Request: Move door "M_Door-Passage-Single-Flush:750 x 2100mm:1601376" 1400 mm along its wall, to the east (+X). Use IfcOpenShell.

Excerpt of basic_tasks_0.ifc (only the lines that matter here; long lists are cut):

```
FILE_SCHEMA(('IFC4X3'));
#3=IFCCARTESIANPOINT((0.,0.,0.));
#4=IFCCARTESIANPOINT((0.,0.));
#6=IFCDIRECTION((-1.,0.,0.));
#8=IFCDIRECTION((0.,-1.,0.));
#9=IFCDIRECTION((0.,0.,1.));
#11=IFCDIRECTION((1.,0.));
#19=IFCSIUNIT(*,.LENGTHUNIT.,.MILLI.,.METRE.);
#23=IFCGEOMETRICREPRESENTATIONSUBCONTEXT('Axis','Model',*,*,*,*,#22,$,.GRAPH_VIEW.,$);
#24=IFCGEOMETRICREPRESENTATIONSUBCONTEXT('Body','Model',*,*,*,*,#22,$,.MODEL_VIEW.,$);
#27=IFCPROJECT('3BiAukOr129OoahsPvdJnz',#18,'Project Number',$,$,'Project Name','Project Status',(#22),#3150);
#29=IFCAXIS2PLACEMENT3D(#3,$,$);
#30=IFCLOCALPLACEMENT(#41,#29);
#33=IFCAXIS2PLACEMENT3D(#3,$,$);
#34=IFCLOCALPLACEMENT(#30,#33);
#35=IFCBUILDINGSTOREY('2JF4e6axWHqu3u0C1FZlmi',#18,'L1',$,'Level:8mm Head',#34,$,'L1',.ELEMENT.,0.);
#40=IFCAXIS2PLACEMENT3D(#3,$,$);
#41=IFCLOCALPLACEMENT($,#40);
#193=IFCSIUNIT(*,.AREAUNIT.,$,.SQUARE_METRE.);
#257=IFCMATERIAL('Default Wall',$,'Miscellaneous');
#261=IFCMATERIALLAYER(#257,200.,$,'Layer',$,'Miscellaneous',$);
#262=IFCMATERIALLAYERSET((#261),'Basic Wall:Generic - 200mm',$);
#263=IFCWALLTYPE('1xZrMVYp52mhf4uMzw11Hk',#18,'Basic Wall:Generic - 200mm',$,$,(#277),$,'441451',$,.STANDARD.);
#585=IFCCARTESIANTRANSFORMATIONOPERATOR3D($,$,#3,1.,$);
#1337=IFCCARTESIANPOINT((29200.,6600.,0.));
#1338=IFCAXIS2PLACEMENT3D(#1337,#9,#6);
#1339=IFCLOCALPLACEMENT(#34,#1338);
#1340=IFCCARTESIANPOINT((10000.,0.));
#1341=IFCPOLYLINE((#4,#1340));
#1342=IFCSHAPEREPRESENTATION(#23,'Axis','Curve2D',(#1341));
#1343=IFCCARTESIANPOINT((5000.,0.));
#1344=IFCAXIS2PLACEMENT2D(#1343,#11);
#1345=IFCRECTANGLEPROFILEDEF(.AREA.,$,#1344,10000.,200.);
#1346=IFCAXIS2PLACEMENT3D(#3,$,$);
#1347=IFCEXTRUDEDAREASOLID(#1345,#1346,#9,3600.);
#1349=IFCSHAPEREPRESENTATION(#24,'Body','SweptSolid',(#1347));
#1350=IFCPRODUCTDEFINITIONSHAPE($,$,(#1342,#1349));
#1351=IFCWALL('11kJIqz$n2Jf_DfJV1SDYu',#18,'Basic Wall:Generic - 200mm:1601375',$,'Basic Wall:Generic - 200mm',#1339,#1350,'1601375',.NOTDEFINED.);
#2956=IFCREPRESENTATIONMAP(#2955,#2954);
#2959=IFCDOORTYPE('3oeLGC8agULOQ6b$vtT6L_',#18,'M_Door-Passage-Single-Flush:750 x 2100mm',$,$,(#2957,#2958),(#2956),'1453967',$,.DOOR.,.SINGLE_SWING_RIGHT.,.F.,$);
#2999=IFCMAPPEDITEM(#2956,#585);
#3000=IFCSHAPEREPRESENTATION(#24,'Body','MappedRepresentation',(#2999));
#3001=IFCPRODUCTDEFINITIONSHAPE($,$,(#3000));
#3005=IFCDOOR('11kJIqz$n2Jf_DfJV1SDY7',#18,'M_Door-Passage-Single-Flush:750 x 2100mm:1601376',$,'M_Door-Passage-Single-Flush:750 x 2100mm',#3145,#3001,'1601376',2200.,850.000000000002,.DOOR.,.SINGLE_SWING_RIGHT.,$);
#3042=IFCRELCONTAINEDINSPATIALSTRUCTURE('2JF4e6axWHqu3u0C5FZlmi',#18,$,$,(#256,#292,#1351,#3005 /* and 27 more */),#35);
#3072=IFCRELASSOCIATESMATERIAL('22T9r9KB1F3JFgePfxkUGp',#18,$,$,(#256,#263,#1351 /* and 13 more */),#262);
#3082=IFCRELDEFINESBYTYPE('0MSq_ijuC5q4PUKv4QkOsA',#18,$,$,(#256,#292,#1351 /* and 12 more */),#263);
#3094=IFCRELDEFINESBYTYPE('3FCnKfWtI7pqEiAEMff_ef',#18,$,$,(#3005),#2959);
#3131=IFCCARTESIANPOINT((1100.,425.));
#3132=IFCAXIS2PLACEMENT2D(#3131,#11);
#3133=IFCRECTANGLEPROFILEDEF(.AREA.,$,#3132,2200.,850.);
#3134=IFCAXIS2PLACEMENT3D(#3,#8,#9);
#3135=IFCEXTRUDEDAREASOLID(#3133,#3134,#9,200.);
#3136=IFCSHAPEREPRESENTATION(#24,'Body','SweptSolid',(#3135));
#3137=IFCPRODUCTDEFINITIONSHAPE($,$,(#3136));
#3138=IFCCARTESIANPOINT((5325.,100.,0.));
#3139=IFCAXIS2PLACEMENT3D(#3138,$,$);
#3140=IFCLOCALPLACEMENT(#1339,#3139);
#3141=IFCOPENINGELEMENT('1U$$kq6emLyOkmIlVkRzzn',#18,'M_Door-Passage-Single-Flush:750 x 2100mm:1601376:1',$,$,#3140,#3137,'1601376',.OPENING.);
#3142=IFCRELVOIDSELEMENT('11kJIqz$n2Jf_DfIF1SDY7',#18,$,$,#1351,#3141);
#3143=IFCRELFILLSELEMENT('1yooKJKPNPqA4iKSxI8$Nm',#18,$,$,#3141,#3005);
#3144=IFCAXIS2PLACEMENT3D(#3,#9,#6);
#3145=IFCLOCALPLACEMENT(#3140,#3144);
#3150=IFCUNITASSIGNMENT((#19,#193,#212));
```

```python
import ifcopenshell
import ifcopenshell.api.geometry
import ifcopenshell.util.placement

model = ifcopenshell.open("basic_tasks_0.ifc")

door = model.by_guid("11kJIqz$n2Jf_DfJV1SDY7")
opening = door.FillsVoids[0].RelatingOpeningElement
wall = opening.VoidsElements[0].RelatingBuildingElement

wall_matrix = ifcopenshell.util.placement.get_local_placement(wall.ObjectPlacement)
shift = wall_matrix[:3, 0] * -1400.0
before = ifcopenshell.util.placement.get_local_placement(door.ObjectPlacement)[:3, 3].copy()

# The door is placed relative to its opening, so it follows when the opening moves.
matrix = ifcopenshell.util.placement.get_local_placement(opening.ObjectPlacement)
matrix[:3, 3] += shift
ifcopenshell.api.geometry.edit_object_placement(
    model, product=opening, matrix=matrix, is_si=False, should_transform_children=True
)

after = ifcopenshell.util.placement.get_local_placement(door.ObjectPlacement)[:3, 3]
print("door moved by", (after - before).round(3) + 0.0)

model.write("basic_tasks_0_updated.ifc")
```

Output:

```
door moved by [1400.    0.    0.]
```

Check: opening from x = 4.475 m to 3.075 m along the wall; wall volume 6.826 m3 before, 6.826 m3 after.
